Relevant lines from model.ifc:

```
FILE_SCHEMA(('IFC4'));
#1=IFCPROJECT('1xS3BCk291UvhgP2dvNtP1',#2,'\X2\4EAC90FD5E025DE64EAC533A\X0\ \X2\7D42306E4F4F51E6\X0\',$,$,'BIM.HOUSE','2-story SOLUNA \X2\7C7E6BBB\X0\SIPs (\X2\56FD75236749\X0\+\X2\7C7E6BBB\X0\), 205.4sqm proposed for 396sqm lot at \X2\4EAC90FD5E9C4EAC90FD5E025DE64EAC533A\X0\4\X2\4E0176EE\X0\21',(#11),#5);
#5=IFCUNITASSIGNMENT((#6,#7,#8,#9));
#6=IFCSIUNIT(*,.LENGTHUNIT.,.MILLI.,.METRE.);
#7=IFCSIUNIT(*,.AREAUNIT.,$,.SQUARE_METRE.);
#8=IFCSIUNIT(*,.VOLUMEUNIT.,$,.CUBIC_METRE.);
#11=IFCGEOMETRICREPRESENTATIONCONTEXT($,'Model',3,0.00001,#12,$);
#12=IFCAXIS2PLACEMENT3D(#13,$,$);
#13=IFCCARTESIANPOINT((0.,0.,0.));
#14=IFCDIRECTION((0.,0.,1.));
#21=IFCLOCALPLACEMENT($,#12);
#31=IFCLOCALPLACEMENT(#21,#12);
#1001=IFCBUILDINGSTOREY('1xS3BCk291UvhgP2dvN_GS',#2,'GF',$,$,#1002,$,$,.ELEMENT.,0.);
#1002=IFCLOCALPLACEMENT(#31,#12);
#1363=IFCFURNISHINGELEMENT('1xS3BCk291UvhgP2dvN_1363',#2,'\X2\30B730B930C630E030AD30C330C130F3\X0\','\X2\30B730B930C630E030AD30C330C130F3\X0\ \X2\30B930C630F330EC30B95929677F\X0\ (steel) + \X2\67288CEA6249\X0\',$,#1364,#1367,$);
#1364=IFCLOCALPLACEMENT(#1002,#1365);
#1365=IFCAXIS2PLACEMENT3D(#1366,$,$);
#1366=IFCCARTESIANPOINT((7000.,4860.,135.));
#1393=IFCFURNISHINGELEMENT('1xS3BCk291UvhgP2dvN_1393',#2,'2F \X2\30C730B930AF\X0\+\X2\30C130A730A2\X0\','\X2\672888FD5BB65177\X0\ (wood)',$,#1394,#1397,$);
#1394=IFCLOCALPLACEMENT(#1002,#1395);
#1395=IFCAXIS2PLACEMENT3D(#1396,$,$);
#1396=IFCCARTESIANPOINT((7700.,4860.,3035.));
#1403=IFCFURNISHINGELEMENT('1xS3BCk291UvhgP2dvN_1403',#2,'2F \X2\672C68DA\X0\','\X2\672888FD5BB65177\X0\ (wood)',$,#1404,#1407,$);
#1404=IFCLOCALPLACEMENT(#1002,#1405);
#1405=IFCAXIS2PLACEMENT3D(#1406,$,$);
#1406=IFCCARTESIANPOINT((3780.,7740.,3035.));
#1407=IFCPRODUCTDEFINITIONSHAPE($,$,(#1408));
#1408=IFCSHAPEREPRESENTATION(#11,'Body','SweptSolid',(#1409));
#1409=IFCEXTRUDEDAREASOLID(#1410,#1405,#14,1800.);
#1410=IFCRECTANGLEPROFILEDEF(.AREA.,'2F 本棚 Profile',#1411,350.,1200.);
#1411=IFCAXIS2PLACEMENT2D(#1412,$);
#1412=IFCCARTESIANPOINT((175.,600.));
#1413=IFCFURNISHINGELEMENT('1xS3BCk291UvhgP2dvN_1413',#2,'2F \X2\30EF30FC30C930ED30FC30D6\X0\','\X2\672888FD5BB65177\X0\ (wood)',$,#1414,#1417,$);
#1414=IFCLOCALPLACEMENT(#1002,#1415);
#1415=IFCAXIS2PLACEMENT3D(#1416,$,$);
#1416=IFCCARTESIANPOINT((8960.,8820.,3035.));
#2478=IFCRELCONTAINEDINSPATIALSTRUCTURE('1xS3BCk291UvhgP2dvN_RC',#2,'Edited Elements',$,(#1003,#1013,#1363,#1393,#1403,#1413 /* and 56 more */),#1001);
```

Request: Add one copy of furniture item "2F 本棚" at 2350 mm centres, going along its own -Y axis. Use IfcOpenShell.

```python
import ifcopenshell
import ifcopenshell.api.geometry
import ifcopenshell.api.root
import ifcopenshell.util.element
import ifcopenshell.util.placement
import ifcopenshell.util.unit

model = ifcopenshell.open("model.ifc")
unit_scale = ifcopenshell.util.unit.calculate_unit_scale(model)


def reuse_history(source, copy):
    """copy_class also copies each property set's owner history, people and application; keep the originals."""
    for rel in copy.IsDefinedBy:
        if rel.is_a("IfcRelDefinesByProperties") and (history := rel.RelatingPropertyDefinition.OwnerHistory):
            rel.RelatingPropertyDefinition.OwnerHistory = source.OwnerHistory
            ifcopenshell.util.element.remove_deep2(model, history)


source = model.by_guid("1xS3BCk291UvhgP2dvN_1403")
base = ifcopenshell.util.placement.get_local_placement(source.ObjectPlacement)
step = -base[:3, 1] * 2.35 / unit_scale

for i in range(1, 2):
    copy = ifcopenshell.api.root.copy_class(model, product=source)
    copy.Representation = ifcopenshell.util.element.copy_deep(
        model, source.Representation, exclude=["IfcGeometricRepresentationContext", "IfcRepresentationMap"]
    )
    reuse_history(source, copy)
    matrix = base.copy()
    matrix[:3, 3] += i * step
    print("added at", matrix[:3, 3].round(3) + 0.0)
    ifcopenshell.api.geometry.edit_object_placement(model, product=copy, matrix=matrix, is_si=False)

model.write("model_updated.ifc")
```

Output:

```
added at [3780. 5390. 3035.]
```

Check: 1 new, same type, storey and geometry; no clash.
